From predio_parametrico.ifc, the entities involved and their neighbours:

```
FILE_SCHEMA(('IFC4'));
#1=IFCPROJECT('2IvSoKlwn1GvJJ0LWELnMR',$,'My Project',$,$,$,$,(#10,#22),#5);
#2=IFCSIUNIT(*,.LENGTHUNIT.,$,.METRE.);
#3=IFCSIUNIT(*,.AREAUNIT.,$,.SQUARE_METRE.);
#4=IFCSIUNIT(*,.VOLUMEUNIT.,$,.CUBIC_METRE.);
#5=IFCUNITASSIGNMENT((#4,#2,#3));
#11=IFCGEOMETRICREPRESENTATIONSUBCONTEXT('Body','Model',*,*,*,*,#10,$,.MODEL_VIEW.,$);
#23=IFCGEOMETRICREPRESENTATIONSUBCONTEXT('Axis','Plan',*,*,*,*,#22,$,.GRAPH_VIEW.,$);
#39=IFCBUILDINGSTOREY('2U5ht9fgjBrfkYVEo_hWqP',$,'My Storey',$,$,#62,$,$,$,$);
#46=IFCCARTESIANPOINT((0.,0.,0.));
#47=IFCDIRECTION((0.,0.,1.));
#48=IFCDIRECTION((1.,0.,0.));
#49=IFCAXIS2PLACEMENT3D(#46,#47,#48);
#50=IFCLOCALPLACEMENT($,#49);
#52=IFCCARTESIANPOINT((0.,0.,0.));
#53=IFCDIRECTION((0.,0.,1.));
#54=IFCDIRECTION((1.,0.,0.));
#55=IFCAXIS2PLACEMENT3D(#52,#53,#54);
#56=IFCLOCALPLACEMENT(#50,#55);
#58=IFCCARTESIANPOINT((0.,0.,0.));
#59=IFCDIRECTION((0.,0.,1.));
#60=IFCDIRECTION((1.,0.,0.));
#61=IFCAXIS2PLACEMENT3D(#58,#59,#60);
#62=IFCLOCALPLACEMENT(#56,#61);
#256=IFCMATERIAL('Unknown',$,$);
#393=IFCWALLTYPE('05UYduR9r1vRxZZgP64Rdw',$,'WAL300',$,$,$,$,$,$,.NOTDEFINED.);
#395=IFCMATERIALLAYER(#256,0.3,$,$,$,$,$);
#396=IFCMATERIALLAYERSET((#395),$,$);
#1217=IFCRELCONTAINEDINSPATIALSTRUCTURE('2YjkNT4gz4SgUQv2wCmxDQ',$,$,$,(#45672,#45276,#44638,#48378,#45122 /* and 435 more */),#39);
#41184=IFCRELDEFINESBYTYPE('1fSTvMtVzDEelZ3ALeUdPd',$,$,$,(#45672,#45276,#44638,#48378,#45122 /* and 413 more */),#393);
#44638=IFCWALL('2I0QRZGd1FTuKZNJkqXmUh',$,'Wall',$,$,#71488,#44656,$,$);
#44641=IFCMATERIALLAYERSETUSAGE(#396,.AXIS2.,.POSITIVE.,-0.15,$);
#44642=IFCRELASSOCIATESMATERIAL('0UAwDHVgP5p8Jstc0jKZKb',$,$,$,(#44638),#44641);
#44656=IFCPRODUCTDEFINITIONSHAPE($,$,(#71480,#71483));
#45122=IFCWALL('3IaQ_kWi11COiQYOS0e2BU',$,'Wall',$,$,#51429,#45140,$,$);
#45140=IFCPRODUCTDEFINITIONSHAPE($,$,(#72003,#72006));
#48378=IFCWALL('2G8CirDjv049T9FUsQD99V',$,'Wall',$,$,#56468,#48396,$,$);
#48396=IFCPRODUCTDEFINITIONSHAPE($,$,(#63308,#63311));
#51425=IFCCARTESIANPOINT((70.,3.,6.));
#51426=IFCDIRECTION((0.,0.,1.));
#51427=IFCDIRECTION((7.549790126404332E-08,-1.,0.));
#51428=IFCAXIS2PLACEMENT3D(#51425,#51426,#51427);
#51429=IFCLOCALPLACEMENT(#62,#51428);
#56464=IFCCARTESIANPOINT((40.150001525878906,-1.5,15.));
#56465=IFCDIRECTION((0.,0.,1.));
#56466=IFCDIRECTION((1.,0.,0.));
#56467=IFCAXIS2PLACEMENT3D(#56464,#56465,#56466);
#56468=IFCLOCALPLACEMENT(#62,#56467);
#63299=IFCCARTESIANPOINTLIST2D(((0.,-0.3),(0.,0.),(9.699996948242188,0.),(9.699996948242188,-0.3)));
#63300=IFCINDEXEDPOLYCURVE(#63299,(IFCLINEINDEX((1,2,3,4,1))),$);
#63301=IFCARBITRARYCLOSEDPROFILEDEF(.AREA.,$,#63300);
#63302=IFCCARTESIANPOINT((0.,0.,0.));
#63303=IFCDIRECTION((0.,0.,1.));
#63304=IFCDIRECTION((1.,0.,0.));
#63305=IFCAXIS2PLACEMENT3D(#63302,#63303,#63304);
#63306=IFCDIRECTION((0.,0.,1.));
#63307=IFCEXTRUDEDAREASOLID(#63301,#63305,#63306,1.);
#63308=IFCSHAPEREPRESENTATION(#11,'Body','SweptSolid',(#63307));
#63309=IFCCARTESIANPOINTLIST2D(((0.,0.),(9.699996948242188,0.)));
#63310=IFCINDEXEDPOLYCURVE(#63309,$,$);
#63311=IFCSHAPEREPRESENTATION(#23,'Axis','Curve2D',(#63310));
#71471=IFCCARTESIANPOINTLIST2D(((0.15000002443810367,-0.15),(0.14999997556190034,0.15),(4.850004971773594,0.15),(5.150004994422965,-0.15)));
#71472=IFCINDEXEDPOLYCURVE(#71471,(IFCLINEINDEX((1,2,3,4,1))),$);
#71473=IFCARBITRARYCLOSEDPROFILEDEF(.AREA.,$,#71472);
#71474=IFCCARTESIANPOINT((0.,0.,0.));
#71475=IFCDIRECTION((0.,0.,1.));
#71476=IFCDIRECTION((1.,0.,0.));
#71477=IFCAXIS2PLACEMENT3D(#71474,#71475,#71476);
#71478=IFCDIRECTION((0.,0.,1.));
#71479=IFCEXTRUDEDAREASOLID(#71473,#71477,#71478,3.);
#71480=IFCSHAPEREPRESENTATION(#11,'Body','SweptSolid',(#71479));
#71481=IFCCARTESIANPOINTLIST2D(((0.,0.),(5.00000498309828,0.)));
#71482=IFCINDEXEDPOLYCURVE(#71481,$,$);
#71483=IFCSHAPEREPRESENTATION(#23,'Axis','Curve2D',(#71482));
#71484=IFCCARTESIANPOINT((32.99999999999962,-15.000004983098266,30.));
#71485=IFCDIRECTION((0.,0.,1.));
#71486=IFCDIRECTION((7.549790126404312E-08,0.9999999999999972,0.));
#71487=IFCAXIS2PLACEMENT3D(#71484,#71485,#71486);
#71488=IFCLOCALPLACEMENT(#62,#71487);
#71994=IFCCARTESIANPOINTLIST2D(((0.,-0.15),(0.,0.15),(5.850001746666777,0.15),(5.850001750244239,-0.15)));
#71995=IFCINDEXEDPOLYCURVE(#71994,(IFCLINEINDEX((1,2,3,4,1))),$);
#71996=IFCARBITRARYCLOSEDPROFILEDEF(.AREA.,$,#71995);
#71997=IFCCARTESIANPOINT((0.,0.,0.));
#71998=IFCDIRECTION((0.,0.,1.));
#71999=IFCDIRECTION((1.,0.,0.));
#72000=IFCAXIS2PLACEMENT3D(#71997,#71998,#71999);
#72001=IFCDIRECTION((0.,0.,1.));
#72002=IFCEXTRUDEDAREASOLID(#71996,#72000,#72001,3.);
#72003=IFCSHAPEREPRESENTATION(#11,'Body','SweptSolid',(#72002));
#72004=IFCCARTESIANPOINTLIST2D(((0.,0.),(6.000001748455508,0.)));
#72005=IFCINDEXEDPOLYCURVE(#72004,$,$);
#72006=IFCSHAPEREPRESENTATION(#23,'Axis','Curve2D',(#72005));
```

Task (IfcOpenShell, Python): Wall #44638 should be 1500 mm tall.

```python
import ifcopenshell
import ifcopenshell.geom
import ifcopenshell.util.representation
import ifcopenshell.util.shape

model = ifcopenshell.open("predio_parametrico.ifc")
settings = ifcopenshell.geom.settings()


def volume(element):
    """Net volume in cubic metres, openings subtracted."""
    shape = ifcopenshell.geom.create_shape(settings, element)
    return ifcopenshell.util.shape.get_volume(shape.geometry)


wall = model.by_id(44638)
before = volume(wall)

body = ifcopenshell.util.representation.get_representation(wall, "Model", "Body")
solid = body.Items[0]
old_height = solid.Depth
solid.Depth = 1.5
after = volume(wall)

print(f"height {old_height:g} -> {solid.Depth:g}, volume {before:.3f} -> {after:.3f} m3")

model.write("predio_parametrico-out.ifc")
```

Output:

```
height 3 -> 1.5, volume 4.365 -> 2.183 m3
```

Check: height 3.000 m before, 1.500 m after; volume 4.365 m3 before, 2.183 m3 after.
